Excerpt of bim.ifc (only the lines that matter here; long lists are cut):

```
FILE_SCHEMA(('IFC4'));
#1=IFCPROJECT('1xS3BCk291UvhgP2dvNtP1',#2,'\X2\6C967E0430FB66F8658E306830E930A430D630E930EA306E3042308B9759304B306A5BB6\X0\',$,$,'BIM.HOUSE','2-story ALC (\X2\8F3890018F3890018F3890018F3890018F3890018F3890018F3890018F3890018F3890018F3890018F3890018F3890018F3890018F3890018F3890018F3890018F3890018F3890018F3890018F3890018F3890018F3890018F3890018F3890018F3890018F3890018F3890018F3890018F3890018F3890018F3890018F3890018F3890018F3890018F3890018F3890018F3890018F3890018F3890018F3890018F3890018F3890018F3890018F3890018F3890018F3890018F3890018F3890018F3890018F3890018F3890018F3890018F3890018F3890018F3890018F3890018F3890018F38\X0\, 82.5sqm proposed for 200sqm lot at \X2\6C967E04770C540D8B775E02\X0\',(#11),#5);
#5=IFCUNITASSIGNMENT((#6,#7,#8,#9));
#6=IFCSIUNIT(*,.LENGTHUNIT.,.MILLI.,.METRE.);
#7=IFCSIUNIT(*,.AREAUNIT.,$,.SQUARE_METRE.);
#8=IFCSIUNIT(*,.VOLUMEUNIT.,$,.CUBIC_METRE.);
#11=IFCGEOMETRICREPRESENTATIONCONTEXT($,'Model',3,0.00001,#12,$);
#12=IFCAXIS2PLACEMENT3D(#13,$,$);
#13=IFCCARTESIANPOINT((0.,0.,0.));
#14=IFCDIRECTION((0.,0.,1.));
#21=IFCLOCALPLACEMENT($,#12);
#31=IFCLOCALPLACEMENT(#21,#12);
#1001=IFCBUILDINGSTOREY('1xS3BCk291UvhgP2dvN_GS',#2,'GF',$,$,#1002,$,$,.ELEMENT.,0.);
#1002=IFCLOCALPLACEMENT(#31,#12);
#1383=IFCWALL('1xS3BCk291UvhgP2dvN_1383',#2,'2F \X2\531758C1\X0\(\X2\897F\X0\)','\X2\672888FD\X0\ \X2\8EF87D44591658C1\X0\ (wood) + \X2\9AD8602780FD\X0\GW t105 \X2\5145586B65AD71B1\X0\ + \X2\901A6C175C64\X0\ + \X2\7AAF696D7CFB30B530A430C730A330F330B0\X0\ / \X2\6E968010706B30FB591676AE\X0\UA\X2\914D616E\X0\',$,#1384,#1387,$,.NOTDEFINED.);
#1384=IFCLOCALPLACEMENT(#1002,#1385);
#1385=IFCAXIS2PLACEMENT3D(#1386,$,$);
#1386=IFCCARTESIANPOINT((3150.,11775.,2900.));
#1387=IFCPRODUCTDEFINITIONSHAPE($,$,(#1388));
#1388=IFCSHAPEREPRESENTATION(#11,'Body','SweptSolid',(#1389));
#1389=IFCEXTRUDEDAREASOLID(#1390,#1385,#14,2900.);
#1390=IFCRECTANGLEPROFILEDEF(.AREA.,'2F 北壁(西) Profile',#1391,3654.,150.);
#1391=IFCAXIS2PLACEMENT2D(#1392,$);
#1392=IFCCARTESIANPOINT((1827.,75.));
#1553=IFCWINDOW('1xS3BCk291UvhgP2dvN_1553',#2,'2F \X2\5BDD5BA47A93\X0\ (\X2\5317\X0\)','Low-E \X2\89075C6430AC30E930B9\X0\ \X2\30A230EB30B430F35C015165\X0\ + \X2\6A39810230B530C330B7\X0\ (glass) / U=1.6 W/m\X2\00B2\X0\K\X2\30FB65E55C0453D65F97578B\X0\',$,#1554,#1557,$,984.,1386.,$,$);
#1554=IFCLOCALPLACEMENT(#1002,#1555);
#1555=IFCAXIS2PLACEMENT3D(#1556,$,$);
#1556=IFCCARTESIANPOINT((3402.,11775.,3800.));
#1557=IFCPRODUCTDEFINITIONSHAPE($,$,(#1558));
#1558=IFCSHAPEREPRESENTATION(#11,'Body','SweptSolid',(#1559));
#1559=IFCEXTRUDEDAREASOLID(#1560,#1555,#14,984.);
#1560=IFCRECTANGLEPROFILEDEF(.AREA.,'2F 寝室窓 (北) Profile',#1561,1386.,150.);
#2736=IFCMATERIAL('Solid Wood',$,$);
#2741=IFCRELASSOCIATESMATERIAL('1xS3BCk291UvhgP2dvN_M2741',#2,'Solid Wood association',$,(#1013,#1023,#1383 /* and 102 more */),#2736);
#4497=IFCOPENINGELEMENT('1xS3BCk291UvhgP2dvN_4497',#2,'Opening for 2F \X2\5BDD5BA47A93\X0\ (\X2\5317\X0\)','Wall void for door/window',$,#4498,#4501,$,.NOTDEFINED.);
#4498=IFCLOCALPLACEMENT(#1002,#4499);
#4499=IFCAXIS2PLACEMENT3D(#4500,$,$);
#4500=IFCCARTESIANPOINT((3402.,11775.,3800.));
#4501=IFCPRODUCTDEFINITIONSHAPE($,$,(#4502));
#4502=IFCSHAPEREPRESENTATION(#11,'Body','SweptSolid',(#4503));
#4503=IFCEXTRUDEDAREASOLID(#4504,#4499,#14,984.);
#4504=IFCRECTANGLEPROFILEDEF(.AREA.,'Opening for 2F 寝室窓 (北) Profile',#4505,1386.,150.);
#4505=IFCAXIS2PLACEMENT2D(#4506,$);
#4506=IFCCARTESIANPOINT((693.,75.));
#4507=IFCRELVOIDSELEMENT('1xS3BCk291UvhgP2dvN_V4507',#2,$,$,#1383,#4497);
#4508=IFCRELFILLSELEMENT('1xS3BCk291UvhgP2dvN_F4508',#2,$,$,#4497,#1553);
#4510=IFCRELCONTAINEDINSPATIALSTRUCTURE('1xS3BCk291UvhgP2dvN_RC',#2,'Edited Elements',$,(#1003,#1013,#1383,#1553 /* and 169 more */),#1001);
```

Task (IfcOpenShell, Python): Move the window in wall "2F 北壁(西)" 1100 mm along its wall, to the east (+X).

```python
import ifcopenshell
import ifcopenshell.api.geometry
import ifcopenshell.util.placement

model = ifcopenshell.open("bim.ifc")

window = model.by_guid("1xS3BCk291UvhgP2dvN_1553")
opening = window.FillsVoids[0].RelatingOpeningElement
wall = opening.VoidsElements[0].RelatingBuildingElement

wall_matrix = ifcopenshell.util.placement.get_local_placement(wall.ObjectPlacement)
shift = wall_matrix[:3, 0] * 1100.0
before = ifcopenshell.util.placement.get_local_placement(window.ObjectPlacement)[:3, 3].copy()

# The window is not placed relative to its opening, so move both.
for product in (opening, window):
    matrix = ifcopenshell.util.placement.get_local_placement(product.ObjectPlacement)
    matrix[:3, 3] += shift
    ifcopenshell.api.geometry.edit_object_placement(model, product=product, matrix=matrix, is_si=False)

after = ifcopenshell.util.placement.get_local_placement(window.ObjectPlacement)[:3, 3]
print("window moved by", (after - before).round(3) + 0.0)

model.write("bim_v2.ifc")
```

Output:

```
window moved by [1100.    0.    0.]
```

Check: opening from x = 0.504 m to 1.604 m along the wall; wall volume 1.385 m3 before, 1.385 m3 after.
